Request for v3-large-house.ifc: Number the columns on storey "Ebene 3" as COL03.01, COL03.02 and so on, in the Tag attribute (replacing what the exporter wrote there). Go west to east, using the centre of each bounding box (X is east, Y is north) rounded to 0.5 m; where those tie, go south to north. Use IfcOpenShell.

First a look at what the model holds.

```python
import ifcopenshell
import ifcopenshell.util.element
import ifcopenshell.util.placement

model = ifcopenshell.open("v3-large-house.ifc")
print(model.schema)
storey = next(s for s in model.by_type("IfcBuildingStorey") if s.Name == "Ebene 3")
columns = [e for e in ifcopenshell.util.element.get_decomposition(storey) if e.is_a("IfcColumn")]
for e in sorted(columns, key=lambda e: e.id()):
    origin = ifcopenshell.util.placement.get_local_placement(e.ObjectPlacement)[:3, 3]
    print(e.id(), e.Tag, e.Name, origin.round(2) + 0.0, sep=" | ")
```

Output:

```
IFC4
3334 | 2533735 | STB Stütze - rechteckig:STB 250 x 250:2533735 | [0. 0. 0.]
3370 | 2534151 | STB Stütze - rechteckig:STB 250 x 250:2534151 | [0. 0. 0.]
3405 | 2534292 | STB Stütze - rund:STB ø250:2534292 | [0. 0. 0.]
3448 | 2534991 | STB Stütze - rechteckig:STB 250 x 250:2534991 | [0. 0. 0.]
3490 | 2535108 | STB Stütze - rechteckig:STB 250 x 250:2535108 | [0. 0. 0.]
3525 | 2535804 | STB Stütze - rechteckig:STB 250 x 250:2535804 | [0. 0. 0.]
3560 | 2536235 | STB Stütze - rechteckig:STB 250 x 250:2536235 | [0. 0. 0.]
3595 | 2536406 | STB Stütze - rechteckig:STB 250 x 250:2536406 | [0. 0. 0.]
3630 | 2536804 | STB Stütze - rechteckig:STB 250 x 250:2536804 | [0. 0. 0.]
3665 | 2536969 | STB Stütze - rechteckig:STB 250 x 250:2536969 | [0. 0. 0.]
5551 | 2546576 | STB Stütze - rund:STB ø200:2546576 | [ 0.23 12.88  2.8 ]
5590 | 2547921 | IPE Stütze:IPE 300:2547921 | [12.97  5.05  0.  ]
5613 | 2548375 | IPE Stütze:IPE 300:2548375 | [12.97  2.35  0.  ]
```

```python
import ifcopenshell
import ifcopenshell.geom
import ifcopenshell.util.element
import ifcopenshell.util.shape

model = ifcopenshell.open("v3-large-house.ifc")
settings = ifcopenshell.geom.settings()
settings.set("use-world-coords", True)


def centre(element):
    shape = ifcopenshell.geom.create_shape(settings, element)
    return ifcopenshell.util.shape.get_bbox_centroid(shape.geometry)


storey = next(s for s in model.by_type("IfcBuildingStorey") if s.Name == "Ebene 3")
columns = [e for e in ifcopenshell.util.element.get_decomposition(storey) if e.is_a("IfcColumn")]

# Insertion points can sit at a corner or the storey origin, so sort by the geometry (in metres).
centres = {e: centre(e) for e in columns}
columns.sort(key=lambda e: (round(centres[e][0] / 0.5), centres[e][1]))

for i, e in enumerate(columns, start=1):
    number = f"COL03.{i:02d}"
    e.Tag = number
    print(e.id(), number)

model.write("v3-large-house_edited.ifc")
```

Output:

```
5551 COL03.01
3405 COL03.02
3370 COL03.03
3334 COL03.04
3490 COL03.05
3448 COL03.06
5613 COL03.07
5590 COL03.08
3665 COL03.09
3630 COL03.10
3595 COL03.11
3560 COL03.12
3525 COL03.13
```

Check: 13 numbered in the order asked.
